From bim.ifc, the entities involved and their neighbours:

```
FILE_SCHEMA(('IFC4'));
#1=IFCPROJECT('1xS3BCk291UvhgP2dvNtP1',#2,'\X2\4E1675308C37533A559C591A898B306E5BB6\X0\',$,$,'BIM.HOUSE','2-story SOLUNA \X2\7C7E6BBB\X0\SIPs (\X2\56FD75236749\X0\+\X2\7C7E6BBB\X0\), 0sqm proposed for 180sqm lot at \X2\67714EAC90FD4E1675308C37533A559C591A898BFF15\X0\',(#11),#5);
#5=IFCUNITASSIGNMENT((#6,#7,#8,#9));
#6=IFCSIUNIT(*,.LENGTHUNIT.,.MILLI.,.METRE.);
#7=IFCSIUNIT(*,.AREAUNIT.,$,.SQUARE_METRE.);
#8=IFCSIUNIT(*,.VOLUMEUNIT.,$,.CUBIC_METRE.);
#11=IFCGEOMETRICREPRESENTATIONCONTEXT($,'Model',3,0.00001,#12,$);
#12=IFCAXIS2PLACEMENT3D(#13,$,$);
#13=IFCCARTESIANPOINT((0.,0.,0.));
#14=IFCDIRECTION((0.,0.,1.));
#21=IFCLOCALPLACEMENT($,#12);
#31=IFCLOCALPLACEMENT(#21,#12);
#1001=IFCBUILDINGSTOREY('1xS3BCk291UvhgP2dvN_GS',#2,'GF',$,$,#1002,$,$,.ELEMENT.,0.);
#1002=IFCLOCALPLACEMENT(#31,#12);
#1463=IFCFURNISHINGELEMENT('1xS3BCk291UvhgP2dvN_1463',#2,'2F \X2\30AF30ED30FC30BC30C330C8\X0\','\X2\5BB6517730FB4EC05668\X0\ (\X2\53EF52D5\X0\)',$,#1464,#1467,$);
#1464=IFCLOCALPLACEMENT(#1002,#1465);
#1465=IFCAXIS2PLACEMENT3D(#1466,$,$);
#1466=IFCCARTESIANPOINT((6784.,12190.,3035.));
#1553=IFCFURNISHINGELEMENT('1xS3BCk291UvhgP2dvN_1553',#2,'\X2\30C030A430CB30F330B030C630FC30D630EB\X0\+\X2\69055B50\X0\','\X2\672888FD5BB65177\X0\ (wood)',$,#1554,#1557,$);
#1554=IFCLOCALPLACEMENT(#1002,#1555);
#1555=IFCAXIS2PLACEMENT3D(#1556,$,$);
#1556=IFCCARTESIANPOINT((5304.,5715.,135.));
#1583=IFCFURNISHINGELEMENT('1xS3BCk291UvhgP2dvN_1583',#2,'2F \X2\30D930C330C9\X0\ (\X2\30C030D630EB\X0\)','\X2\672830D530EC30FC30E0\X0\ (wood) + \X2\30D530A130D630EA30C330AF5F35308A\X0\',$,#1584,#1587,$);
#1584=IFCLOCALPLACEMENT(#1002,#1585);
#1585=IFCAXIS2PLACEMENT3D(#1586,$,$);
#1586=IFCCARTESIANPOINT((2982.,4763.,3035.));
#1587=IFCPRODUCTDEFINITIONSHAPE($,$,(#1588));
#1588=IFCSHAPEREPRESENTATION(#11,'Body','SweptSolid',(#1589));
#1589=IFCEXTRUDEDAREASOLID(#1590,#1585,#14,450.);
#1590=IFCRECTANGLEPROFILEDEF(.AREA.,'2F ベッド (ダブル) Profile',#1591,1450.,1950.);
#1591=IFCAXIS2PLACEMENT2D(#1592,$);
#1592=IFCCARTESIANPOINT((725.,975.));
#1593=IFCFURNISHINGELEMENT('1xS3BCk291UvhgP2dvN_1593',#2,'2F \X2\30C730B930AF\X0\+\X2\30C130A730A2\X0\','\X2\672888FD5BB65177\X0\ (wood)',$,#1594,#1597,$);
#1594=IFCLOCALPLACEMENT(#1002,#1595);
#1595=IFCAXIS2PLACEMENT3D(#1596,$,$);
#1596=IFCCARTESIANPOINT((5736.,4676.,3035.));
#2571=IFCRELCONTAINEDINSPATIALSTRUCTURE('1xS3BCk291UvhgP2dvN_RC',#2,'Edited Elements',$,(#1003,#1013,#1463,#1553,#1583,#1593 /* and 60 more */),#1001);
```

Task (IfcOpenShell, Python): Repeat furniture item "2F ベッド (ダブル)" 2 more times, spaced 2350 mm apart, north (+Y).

```python
import numpy as np
import ifcopenshell
import ifcopenshell.api.geometry
import ifcopenshell.api.root
import ifcopenshell.util.element
import ifcopenshell.util.placement
import ifcopenshell.util.unit

model = ifcopenshell.open("bim.ifc")
unit_scale = ifcopenshell.util.unit.calculate_unit_scale(model)


def reuse_history(source, copy):
    """copy_class also copies each property set's owner history, people and application; keep the originals."""
    for rel in copy.IsDefinedBy:
        if rel.is_a("IfcRelDefinesByProperties") and (history := rel.RelatingPropertyDefinition.OwnerHistory):
            rel.RelatingPropertyDefinition.OwnerHistory = source.OwnerHistory
            ifcopenshell.util.element.remove_deep2(model, history)


source = model.by_id(1583)
base = ifcopenshell.util.placement.get_local_placement(source.ObjectPlacement)
step = np.array([0.0, 1.0, 0.0]) * 2.35 / unit_scale

for i in range(1, 3):
    copy = ifcopenshell.api.root.copy_class(model, product=source)
    copy.Representation = ifcopenshell.util.element.copy_deep(
        model, source.Representation, exclude=["IfcGeometricRepresentationContext", "IfcRepresentationMap"]
    )
    reuse_history(source, copy)
    matrix = base.copy()
    matrix[:3, 3] += i * step
    print("added at", matrix[:3, 3].round(3) + 0.0)
    ifcopenshell.api.geometry.edit_object_placement(model, product=copy, matrix=matrix, is_si=False)

model.write("bim-out.ifc")
```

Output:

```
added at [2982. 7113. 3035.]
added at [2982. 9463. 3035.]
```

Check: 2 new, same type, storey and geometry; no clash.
